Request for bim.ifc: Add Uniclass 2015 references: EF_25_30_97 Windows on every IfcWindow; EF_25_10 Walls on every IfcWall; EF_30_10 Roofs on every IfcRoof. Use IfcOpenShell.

First a look at what the model holds.

```python
import ifcopenshell

model = ifcopenshell.open("bim.ifc")
print(model.schema)
print("classifications:", [c.Name for c in model.by_type("IfcClassification")])
for ifc_class in ("IfcDoor", "IfcRoof", "IfcStair", "IfcWall", "IfcWindow"):
    print(ifc_class, len(model.by_type(ifc_class)))
```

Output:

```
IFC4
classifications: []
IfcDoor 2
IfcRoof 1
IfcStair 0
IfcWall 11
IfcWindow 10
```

```python
import ifcopenshell
import ifcopenshell.api.classification

model = ifcopenshell.open("bim.ifc")

system = ifcopenshell.api.classification.add_classification(model, classification="Uniclass 2015")

codes = {
    "IfcWindow": ("EF_25_30_97", "Windows"),
    "IfcWall": ("EF_25_10", "Walls"),
    "IfcRoof": ("EF_30_10", "Roofs"),
}
for ifc_class, (code, name) in codes.items():
    products = model.by_type(ifc_class)
    ifcopenshell.api.classification.add_reference(
        model, products=products, classification=system, identification=code, name=name
    )
    print(code, len(products))

model.write("bim-out.ifc")
```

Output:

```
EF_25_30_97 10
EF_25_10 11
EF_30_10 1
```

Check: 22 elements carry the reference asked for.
